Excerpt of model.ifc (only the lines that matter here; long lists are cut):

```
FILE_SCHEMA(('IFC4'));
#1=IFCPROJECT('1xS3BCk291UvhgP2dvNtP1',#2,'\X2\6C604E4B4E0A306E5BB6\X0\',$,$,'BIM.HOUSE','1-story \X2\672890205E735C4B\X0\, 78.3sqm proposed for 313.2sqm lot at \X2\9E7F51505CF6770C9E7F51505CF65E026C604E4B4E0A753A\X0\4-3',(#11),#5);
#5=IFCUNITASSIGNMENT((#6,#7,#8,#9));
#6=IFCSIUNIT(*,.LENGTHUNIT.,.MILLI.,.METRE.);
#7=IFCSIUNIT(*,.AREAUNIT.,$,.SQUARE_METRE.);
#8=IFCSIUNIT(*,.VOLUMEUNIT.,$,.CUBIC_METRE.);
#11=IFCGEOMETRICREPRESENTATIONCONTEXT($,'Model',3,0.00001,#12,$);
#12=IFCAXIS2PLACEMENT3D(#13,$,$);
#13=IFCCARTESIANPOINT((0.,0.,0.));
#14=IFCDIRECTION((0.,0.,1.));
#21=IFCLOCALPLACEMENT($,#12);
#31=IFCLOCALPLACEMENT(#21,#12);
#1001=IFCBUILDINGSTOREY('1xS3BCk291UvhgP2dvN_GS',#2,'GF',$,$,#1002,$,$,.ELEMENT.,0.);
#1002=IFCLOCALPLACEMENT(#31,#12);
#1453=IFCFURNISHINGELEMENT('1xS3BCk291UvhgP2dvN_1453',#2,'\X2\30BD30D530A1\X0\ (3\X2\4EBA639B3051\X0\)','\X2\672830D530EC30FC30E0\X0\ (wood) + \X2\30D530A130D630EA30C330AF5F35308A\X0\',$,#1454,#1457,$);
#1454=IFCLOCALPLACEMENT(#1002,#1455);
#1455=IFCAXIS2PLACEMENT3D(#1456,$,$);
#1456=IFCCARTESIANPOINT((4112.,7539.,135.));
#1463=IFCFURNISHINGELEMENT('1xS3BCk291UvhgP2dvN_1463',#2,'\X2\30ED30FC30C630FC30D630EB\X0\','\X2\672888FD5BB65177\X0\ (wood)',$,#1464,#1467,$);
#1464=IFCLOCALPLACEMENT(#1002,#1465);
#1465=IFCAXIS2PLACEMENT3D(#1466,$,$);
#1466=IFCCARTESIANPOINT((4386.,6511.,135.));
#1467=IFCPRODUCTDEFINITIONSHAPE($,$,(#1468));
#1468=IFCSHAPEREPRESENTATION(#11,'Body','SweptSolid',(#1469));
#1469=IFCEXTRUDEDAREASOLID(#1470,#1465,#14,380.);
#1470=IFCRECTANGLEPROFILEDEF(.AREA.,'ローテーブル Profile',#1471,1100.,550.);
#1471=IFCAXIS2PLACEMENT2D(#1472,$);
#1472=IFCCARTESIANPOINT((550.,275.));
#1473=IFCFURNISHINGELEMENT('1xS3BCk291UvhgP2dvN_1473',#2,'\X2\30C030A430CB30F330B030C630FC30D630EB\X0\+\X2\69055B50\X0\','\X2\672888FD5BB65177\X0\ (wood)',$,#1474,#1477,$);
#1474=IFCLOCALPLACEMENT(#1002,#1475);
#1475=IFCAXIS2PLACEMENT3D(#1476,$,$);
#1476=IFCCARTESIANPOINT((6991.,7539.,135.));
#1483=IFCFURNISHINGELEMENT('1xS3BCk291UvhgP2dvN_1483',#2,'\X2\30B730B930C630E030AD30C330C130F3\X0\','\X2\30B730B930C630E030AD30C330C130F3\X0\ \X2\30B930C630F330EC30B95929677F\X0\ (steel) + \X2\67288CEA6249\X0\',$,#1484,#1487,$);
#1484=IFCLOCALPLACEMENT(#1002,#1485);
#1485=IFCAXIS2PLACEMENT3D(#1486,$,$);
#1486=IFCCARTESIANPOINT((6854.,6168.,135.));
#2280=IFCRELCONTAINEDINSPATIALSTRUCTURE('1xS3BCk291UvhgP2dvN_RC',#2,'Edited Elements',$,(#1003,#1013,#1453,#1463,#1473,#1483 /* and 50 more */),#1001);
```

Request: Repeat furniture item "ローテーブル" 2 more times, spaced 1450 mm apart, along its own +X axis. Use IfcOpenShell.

```python
import ifcopenshell
import ifcopenshell.api.geometry
import ifcopenshell.api.root
import ifcopenshell.util.element
import ifcopenshell.util.placement
import ifcopenshell.util.unit

model = ifcopenshell.open("model.ifc")
unit_scale = ifcopenshell.util.unit.calculate_unit_scale(model)


def reuse_history(source, copy):
    """copy_class also copies each property set's owner history, people and application; keep the originals."""
    for rel in copy.IsDefinedBy:
        if rel.is_a("IfcRelDefinesByProperties") and (history := rel.RelatingPropertyDefinition.OwnerHistory):
            rel.RelatingPropertyDefinition.OwnerHistory = source.OwnerHistory
            ifcopenshell.util.element.remove_deep2(model, history)


source = model.by_id(1463)
base = ifcopenshell.util.placement.get_local_placement(source.ObjectPlacement)
step = base[:3, 0] * 1.45 / unit_scale

for i in range(1, 3):
    copy = ifcopenshell.api.root.copy_class(model, product=source)
    copy.Representation = ifcopenshell.util.element.copy_deep(
        model, source.Representation, exclude=["IfcGeometricRepresentationContext", "IfcRepresentationMap"]
    )
    reuse_history(source, copy)
    matrix = base.copy()
    matrix[:3, 3] += i * step
    print("added at", matrix[:3, 3].round(3) + 0.0)
    ifcopenshell.api.geometry.edit_object_placement(model, product=copy, matrix=matrix, is_si=False)

model.write("model_updated.ifc")
```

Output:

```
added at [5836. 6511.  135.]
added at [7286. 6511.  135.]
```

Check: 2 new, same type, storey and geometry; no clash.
